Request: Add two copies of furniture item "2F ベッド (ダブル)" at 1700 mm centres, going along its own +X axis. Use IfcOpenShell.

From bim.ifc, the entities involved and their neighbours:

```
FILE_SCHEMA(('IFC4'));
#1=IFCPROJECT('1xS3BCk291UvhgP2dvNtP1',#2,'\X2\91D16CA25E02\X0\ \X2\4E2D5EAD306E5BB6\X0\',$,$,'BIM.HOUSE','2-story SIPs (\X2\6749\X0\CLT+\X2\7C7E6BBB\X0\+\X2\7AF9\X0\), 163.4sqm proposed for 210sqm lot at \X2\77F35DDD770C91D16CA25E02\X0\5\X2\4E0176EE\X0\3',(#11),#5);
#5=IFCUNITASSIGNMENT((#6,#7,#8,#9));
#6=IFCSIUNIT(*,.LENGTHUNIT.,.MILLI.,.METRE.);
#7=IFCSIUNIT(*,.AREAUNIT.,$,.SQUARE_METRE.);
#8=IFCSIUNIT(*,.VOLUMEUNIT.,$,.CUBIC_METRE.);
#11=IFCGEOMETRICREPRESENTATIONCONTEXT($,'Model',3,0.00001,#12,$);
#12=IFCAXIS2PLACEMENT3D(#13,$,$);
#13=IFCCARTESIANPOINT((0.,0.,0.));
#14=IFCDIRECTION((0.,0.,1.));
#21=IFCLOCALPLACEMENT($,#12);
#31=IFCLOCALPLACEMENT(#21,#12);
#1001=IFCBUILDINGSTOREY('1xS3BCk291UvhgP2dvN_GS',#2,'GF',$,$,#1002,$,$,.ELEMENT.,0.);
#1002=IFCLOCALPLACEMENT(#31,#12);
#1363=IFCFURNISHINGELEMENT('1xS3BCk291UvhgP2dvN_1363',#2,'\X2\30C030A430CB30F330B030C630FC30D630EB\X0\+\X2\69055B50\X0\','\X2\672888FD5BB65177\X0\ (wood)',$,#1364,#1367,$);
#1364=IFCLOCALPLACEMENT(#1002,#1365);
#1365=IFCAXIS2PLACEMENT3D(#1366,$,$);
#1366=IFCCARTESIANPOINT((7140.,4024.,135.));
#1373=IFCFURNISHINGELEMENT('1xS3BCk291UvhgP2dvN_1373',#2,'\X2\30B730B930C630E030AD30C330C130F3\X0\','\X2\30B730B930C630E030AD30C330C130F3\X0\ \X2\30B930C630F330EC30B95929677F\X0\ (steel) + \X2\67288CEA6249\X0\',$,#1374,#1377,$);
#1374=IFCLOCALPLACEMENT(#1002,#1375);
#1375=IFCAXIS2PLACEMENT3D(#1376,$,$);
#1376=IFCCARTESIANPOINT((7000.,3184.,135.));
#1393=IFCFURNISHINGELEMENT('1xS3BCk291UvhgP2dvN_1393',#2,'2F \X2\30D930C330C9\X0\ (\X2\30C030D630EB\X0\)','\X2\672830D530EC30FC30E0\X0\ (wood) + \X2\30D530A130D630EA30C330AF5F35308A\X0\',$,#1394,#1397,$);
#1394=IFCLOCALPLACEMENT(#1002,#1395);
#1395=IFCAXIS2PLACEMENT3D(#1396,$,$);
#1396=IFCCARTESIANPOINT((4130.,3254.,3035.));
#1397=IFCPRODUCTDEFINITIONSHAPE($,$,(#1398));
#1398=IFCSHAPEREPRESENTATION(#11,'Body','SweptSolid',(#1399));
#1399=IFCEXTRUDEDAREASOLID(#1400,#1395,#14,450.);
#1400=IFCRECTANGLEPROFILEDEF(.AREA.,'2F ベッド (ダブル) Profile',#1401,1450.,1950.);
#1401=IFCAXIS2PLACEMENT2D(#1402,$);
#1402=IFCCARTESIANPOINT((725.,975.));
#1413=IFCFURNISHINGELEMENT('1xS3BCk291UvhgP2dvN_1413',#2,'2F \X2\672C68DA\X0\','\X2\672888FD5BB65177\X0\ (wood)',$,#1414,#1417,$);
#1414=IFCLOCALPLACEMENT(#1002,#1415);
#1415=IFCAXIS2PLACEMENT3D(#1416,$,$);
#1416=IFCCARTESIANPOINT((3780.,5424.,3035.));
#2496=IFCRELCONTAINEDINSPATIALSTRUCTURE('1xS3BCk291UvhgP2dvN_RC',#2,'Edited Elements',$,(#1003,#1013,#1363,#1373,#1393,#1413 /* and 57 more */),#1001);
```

```python
import ifcopenshell
import ifcopenshell.api.geometry
import ifcopenshell.api.root
import ifcopenshell.util.element
import ifcopenshell.util.placement

model = ifcopenshell.open("bim.ifc")


def reuse_history(source, copy):
    """copy_class also copies each property set's owner history, people and application; keep the originals."""
    for rel in copy.IsDefinedBy:
        if rel.is_a("IfcRelDefinesByProperties") and (history := rel.RelatingPropertyDefinition.OwnerHistory):
            rel.RelatingPropertyDefinition.OwnerHistory = source.OwnerHistory
            ifcopenshell.util.element.remove_deep2(model, history)


source = model.by_guid("1xS3BCk291UvhgP2dvN_1393")
base = ifcopenshell.util.placement.get_local_placement(source.ObjectPlacement)
step = base[:3, 0] * 1700.0

for i in range(1, 3):
    copy = ifcopenshell.api.root.copy_class(model, product=source)
    copy.Representation = ifcopenshell.util.element.copy_deep(
        model, source.Representation, exclude=["IfcGeometricRepresentationContext", "IfcRepresentationMap"]
    )
    reuse_history(source, copy)
    matrix = base.copy()
    matrix[:3, 3] += i * step
    print("added at", matrix[:3, 3].round(3) + 0.0)
    ifcopenshell.api.geometry.edit_object_placement(model, product=copy, matrix=matrix, is_si=False)

model.write("bim_v2.ifc")
```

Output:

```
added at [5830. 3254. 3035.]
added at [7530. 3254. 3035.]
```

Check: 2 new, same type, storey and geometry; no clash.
